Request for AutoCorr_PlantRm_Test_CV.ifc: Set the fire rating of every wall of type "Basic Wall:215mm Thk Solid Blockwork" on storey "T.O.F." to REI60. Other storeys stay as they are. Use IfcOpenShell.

First a look at what the model holds.

```python
import ifcopenshell
import ifcopenshell.util.element

model = ifcopenshell.open("AutoCorr_PlantRm_Test_CV.ifc")
print(model.schema)
storey = next(s for s in model.by_type("IfcBuildingStorey") if s.Name == "T.O.F.")
walls = [e for e in ifcopenshell.util.element.get_decomposition(storey) if e.is_a("IfcWall")]
seen = {}
for e in walls:
    element_type = ifcopenshell.util.element.get_type(e)
    key = (element_type.Name if element_type != e and element_type else None, ifcopenshell.util.element.get_pset(e, "Pset_WallCommon", "FireRating"))
    seen[key] = seen.get(key, 0) + 1
for (name, value), count in sorted(seen.items(), key=str):
    print(count, "x", name, "|", value)
```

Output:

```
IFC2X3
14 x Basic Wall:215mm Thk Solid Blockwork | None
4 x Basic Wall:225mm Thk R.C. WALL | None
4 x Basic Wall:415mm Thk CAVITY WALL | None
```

```python
import ifcopenshell
import ifcopenshell.api.pset
import ifcopenshell.util.element

model = ifcopenshell.open("AutoCorr_PlantRm_Test_CV.ifc")

storey = next(s for s in model.by_type("IfcBuildingStorey") if s.Name == "T.O.F.")
walls = [e for e in ifcopenshell.util.element.get_decomposition(storey) if e.is_a("IfcWall")]

count = 0
for e in walls:
    element_type = ifcopenshell.util.element.get_type(e)
    if element_type in (None, e) or element_type.Name != "Basic Wall:215mm Thk Solid Blockwork":
        continue
    # add_pset returns the element's existing set when there is one.
    pset = ifcopenshell.api.pset.add_pset(model, product=e, name="Pset_WallCommon")
    ifcopenshell.api.pset.edit_pset(model, pset=pset, properties={"FireRating": "REI60"})
    count += 1

print(count, "walls updated")

model.write("AutoCorr_PlantRm_Test_CV_updated.ifc")
```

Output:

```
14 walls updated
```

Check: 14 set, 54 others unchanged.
